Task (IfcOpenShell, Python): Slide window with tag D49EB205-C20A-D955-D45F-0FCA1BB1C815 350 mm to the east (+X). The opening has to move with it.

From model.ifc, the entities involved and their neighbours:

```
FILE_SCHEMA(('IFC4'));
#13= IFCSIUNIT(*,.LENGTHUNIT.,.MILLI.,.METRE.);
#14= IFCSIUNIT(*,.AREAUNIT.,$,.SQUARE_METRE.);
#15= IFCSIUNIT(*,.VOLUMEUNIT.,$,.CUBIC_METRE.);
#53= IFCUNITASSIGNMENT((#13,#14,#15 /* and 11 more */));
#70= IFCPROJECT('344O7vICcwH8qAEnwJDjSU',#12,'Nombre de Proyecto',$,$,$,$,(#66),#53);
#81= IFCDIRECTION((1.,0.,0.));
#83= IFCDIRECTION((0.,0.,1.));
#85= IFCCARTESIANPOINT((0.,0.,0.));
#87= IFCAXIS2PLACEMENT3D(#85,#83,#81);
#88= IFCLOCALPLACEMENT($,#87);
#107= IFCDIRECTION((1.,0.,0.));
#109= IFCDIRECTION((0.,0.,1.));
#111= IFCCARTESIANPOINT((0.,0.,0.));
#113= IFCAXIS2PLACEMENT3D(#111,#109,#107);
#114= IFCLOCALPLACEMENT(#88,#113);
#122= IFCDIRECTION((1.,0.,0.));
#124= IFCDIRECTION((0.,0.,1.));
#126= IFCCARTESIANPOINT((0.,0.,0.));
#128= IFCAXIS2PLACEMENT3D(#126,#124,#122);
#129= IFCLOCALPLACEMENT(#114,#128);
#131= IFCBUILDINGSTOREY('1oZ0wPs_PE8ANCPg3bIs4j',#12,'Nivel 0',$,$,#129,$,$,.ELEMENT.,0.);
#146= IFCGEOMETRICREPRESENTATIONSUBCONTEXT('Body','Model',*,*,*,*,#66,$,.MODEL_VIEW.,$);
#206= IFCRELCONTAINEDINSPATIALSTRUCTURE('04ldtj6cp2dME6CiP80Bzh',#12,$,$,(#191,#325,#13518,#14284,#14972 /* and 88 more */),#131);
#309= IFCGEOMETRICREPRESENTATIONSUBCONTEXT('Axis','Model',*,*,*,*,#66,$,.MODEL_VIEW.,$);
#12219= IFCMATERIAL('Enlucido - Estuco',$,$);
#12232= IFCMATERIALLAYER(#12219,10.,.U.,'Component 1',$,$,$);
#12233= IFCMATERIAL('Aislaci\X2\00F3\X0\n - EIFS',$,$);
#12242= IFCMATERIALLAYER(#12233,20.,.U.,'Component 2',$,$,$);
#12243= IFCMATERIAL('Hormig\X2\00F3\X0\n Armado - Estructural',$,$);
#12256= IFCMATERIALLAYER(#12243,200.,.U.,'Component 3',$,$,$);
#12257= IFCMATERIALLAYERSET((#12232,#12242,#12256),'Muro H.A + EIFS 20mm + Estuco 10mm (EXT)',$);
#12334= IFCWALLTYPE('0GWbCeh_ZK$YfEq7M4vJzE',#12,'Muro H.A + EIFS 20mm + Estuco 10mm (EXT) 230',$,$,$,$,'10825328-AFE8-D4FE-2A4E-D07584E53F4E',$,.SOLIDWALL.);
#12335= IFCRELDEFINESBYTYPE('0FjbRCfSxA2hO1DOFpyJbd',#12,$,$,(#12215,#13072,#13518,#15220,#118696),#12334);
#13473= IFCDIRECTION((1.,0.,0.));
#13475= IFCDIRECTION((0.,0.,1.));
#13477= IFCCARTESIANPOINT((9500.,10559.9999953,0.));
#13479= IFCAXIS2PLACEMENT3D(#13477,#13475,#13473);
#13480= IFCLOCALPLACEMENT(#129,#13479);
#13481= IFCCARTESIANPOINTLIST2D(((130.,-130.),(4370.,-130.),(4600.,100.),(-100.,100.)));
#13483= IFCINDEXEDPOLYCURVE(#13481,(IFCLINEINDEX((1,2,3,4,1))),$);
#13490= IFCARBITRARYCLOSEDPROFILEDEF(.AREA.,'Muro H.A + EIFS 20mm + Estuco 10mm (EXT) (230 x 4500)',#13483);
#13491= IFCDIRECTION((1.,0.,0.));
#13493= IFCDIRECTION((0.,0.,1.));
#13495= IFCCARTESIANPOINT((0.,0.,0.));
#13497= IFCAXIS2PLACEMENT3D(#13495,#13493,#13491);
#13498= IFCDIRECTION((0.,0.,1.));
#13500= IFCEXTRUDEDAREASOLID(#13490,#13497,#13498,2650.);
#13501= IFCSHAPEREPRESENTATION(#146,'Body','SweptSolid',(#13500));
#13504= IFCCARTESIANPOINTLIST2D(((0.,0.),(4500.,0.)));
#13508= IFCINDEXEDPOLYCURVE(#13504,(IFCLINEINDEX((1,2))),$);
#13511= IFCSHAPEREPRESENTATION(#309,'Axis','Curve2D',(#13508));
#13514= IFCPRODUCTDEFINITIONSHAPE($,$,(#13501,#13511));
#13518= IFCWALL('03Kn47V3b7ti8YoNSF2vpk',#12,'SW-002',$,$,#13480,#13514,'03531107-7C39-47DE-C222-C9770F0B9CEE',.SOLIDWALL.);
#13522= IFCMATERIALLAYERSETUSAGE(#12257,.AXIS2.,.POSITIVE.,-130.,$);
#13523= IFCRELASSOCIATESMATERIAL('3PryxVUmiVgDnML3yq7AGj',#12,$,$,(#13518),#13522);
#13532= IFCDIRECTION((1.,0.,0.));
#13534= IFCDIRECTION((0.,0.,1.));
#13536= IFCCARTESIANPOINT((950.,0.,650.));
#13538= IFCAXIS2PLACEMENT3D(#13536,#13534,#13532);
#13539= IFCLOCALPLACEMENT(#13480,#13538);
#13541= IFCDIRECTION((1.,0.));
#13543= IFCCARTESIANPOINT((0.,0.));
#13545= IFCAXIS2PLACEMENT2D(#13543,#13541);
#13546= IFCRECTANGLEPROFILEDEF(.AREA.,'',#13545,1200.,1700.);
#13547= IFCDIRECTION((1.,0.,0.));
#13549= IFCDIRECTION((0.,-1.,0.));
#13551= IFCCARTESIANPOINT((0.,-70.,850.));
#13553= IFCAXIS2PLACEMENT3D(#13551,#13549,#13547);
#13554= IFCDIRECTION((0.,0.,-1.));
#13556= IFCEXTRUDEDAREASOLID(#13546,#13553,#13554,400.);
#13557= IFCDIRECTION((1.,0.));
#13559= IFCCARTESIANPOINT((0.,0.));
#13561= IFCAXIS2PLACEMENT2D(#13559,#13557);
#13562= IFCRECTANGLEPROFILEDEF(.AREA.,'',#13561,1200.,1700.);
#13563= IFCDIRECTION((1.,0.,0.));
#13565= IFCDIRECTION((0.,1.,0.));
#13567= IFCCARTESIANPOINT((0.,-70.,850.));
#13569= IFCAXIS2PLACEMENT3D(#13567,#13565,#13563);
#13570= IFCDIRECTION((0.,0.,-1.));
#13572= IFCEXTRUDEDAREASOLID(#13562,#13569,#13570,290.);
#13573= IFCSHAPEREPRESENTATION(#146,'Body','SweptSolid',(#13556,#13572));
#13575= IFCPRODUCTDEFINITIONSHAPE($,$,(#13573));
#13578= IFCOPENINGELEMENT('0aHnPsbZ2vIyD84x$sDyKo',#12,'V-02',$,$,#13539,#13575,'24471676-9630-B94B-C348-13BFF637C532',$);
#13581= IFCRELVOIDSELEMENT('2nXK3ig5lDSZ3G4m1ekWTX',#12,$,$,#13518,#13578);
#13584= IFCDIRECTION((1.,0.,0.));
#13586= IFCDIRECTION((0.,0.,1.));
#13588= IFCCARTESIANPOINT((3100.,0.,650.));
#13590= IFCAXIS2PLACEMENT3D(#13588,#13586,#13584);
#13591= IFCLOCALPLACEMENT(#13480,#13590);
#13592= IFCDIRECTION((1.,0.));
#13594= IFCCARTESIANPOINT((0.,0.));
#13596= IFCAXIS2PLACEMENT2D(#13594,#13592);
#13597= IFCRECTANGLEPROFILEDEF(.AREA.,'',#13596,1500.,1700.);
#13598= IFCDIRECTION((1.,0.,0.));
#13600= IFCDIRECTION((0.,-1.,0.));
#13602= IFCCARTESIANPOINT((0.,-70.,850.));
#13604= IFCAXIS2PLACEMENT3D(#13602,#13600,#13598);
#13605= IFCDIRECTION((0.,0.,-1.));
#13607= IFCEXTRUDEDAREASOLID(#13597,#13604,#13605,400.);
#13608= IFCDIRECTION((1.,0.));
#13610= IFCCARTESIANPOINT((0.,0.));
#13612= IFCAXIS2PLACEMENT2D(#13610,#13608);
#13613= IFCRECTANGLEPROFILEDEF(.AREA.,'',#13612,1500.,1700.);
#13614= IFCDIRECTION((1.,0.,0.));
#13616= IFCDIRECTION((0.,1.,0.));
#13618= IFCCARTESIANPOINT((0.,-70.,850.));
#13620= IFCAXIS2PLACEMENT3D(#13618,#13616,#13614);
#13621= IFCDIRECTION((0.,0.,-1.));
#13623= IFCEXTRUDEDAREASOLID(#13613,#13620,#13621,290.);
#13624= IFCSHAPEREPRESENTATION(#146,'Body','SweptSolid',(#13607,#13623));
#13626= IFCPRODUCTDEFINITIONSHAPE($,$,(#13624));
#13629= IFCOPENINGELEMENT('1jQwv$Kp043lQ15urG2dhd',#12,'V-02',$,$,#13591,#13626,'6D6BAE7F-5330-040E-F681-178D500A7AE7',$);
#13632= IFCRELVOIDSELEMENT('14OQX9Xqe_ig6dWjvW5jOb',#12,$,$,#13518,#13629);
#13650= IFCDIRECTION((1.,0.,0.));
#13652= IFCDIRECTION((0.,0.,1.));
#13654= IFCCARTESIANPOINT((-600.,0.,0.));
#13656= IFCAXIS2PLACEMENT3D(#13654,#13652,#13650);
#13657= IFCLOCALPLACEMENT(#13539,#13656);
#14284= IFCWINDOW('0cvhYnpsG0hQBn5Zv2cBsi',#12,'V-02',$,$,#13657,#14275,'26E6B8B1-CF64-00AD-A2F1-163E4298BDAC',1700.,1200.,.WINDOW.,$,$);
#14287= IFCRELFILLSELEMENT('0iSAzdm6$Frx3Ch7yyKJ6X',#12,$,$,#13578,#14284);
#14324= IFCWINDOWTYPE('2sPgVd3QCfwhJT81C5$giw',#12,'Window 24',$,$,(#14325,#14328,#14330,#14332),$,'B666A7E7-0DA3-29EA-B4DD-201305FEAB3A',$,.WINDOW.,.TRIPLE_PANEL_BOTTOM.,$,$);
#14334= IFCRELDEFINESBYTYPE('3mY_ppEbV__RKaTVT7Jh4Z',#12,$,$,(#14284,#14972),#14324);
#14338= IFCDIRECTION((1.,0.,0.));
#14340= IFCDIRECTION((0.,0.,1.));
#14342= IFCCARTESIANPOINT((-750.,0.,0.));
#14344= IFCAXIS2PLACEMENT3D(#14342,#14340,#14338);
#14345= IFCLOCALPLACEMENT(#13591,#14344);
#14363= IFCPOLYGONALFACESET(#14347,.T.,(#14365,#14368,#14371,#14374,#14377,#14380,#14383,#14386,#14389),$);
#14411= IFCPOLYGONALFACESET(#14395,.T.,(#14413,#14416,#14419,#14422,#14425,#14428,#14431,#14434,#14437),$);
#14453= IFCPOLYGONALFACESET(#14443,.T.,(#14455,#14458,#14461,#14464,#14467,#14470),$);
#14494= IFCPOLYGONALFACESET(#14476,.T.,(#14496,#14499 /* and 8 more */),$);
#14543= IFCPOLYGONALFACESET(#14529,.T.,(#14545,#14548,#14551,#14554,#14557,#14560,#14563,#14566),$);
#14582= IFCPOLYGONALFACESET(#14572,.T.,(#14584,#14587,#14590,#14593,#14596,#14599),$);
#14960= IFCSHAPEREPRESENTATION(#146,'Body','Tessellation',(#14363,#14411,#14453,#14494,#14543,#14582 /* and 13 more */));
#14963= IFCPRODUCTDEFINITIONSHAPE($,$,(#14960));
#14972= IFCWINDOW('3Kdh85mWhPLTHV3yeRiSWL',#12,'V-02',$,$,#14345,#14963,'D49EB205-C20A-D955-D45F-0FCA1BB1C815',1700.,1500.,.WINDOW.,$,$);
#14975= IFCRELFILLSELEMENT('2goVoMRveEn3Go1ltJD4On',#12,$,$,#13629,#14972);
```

```python
import ifcopenshell
import ifcopenshell.api.geometry
import ifcopenshell.util.placement

model = ifcopenshell.open("model.ifc")

window = model.by_guid("3Kdh85mWhPLTHV3yeRiSWL")
opening = window.FillsVoids[0].RelatingOpeningElement
wall = opening.VoidsElements[0].RelatingBuildingElement

wall_matrix = ifcopenshell.util.placement.get_local_placement(wall.ObjectPlacement)
shift = wall_matrix[:3, 0] * 350.0
before = ifcopenshell.util.placement.get_local_placement(window.ObjectPlacement)[:3, 3].copy()

# The window is placed relative to its opening, so it follows when the opening moves.
matrix = ifcopenshell.util.placement.get_local_placement(opening.ObjectPlacement)
matrix[:3, 3] += shift
ifcopenshell.api.geometry.edit_object_placement(
    model, product=opening, matrix=matrix, is_si=False, should_transform_children=True
)

after = ifcopenshell.util.placement.get_local_placement(window.ObjectPlacement)[:3, 3]
print("window moved by", (after - before).round(3) + 0.0)

model.write("model_rev.ifc")
```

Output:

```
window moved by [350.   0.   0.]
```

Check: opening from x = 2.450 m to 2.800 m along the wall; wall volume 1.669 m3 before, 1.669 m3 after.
